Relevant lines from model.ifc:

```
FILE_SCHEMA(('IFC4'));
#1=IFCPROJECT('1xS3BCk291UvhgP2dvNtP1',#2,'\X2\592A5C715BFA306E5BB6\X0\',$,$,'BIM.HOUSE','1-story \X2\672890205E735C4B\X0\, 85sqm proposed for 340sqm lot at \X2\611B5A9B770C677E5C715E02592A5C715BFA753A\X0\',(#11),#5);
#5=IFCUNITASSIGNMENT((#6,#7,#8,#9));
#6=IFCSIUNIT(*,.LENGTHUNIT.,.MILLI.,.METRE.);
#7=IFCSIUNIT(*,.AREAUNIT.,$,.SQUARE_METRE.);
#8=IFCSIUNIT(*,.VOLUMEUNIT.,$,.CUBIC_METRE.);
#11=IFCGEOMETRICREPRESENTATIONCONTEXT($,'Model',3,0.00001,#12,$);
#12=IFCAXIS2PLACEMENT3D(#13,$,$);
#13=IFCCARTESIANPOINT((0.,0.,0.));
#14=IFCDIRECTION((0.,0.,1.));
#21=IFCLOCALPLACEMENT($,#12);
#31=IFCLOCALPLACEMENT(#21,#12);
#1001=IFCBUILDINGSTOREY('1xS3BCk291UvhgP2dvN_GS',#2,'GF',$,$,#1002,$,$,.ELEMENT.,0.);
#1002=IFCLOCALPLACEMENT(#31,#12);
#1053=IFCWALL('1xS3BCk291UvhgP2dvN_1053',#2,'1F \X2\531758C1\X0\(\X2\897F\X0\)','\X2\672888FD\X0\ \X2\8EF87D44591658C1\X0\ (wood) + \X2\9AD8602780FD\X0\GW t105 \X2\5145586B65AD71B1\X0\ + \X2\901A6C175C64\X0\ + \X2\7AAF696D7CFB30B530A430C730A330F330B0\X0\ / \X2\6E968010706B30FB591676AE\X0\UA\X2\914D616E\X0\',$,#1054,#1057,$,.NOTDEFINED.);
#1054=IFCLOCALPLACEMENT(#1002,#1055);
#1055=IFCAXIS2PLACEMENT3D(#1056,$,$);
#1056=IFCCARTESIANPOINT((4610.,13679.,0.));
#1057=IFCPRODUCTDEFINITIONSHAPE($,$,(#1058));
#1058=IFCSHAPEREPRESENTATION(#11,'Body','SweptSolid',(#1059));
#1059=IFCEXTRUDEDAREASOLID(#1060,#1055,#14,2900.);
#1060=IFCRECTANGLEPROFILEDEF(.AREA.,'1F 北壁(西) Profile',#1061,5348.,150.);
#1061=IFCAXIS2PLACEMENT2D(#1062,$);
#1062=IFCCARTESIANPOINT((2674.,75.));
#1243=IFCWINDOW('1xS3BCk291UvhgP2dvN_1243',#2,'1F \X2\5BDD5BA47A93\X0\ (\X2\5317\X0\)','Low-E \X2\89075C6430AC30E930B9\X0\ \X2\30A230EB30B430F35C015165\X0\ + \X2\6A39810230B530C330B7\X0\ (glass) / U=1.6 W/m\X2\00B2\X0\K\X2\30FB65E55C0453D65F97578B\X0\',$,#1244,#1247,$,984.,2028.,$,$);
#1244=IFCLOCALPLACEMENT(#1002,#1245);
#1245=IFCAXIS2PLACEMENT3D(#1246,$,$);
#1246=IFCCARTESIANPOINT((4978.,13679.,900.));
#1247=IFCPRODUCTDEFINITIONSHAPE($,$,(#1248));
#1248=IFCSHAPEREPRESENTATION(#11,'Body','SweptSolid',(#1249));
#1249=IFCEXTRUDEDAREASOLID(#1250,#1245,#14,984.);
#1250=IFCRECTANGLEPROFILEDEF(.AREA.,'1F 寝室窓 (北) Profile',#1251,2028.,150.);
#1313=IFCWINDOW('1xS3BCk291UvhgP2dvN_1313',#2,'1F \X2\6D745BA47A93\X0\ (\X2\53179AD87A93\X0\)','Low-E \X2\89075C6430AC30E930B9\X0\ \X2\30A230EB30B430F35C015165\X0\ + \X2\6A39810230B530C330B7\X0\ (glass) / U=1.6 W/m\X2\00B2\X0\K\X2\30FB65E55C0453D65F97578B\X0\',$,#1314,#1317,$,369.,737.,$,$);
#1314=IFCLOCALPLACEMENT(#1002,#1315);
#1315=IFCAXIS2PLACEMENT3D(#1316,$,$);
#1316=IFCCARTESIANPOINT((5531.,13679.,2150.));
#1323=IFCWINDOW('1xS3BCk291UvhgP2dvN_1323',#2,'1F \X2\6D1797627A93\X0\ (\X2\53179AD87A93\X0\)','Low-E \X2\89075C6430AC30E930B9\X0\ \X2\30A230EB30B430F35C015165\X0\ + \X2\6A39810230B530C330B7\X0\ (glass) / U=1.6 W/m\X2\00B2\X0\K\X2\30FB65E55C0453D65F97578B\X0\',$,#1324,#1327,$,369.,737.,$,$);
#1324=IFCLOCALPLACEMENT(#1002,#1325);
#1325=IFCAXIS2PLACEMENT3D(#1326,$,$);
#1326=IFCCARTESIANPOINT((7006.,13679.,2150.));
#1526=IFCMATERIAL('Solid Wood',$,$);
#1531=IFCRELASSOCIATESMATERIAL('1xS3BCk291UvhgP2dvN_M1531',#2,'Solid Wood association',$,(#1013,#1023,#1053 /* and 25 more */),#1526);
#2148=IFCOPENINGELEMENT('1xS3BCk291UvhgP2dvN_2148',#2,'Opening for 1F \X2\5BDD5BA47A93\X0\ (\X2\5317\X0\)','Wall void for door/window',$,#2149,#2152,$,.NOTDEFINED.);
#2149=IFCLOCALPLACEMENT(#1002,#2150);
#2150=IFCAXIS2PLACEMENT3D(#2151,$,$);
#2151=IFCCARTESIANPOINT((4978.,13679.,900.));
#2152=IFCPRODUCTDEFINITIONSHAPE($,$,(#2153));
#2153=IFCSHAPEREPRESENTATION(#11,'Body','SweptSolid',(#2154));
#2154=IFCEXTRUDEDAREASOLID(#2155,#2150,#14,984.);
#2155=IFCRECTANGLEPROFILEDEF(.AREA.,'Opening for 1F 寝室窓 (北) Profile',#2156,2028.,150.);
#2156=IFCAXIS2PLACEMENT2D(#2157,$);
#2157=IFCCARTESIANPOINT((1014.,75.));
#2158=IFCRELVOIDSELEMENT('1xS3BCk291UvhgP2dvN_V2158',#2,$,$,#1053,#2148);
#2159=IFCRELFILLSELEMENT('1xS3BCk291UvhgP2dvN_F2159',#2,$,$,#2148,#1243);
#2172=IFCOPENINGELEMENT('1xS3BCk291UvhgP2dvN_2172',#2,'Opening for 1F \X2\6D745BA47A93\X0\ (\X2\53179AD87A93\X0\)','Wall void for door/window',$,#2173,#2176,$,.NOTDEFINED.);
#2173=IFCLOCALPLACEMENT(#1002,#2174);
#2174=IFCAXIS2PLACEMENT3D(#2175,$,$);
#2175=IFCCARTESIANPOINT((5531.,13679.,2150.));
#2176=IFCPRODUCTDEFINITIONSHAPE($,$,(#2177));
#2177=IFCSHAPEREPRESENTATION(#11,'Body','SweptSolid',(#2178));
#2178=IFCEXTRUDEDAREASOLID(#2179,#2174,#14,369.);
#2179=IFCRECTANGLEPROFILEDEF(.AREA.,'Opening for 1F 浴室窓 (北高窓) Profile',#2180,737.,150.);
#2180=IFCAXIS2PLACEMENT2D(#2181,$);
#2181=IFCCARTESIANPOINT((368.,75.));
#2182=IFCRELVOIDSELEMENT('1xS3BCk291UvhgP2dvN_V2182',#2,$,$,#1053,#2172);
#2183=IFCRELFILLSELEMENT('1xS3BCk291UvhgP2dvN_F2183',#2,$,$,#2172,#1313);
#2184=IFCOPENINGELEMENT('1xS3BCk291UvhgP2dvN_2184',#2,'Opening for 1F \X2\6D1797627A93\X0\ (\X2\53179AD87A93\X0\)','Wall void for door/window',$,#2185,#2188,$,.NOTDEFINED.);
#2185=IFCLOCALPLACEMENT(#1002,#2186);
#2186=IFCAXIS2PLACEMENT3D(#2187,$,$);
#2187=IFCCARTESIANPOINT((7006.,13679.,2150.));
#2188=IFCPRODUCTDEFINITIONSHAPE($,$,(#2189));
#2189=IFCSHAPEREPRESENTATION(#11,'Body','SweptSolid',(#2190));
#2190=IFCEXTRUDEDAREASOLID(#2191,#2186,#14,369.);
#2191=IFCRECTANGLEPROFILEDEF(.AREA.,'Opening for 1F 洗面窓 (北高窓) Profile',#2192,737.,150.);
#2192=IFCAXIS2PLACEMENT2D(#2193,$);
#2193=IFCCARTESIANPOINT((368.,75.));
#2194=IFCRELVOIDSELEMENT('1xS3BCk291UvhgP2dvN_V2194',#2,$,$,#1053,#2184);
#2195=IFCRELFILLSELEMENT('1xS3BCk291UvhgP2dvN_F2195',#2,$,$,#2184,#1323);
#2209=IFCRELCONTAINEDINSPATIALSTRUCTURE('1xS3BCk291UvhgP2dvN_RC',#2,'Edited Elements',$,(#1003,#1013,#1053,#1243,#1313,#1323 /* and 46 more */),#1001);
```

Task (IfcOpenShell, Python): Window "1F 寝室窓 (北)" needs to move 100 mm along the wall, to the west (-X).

```python
import ifcopenshell
import ifcopenshell.api.geometry
import ifcopenshell.util.placement
import ifcopenshell.util.unit

model = ifcopenshell.open("model.ifc")
unit_scale = ifcopenshell.util.unit.calculate_unit_scale(model)

window = model.by_guid("1xS3BCk291UvhgP2dvN_1243")
opening = window.FillsVoids[0].RelatingOpeningElement
wall = opening.VoidsElements[0].RelatingBuildingElement

wall_matrix = ifcopenshell.util.placement.get_local_placement(wall.ObjectPlacement)
shift = wall_matrix[:3, 0] * -0.1 / unit_scale
before = ifcopenshell.util.placement.get_local_placement(window.ObjectPlacement)[:3, 3].copy()

# The window is not placed relative to its opening, so move both.
for product in (opening, window):
    matrix = ifcopenshell.util.placement.get_local_placement(product.ObjectPlacement)
    matrix[:3, 3] += shift
    ifcopenshell.api.geometry.edit_object_placement(model, product=product, matrix=matrix, is_si=False)

after = ifcopenshell.util.placement.get_local_placement(window.ObjectPlacement)[:3, 3]
print("window moved by", (after - before).round(3) + 0.0)

model.write("model_edited.ifc")
```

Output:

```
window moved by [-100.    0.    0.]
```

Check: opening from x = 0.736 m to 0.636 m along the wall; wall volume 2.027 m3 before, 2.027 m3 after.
